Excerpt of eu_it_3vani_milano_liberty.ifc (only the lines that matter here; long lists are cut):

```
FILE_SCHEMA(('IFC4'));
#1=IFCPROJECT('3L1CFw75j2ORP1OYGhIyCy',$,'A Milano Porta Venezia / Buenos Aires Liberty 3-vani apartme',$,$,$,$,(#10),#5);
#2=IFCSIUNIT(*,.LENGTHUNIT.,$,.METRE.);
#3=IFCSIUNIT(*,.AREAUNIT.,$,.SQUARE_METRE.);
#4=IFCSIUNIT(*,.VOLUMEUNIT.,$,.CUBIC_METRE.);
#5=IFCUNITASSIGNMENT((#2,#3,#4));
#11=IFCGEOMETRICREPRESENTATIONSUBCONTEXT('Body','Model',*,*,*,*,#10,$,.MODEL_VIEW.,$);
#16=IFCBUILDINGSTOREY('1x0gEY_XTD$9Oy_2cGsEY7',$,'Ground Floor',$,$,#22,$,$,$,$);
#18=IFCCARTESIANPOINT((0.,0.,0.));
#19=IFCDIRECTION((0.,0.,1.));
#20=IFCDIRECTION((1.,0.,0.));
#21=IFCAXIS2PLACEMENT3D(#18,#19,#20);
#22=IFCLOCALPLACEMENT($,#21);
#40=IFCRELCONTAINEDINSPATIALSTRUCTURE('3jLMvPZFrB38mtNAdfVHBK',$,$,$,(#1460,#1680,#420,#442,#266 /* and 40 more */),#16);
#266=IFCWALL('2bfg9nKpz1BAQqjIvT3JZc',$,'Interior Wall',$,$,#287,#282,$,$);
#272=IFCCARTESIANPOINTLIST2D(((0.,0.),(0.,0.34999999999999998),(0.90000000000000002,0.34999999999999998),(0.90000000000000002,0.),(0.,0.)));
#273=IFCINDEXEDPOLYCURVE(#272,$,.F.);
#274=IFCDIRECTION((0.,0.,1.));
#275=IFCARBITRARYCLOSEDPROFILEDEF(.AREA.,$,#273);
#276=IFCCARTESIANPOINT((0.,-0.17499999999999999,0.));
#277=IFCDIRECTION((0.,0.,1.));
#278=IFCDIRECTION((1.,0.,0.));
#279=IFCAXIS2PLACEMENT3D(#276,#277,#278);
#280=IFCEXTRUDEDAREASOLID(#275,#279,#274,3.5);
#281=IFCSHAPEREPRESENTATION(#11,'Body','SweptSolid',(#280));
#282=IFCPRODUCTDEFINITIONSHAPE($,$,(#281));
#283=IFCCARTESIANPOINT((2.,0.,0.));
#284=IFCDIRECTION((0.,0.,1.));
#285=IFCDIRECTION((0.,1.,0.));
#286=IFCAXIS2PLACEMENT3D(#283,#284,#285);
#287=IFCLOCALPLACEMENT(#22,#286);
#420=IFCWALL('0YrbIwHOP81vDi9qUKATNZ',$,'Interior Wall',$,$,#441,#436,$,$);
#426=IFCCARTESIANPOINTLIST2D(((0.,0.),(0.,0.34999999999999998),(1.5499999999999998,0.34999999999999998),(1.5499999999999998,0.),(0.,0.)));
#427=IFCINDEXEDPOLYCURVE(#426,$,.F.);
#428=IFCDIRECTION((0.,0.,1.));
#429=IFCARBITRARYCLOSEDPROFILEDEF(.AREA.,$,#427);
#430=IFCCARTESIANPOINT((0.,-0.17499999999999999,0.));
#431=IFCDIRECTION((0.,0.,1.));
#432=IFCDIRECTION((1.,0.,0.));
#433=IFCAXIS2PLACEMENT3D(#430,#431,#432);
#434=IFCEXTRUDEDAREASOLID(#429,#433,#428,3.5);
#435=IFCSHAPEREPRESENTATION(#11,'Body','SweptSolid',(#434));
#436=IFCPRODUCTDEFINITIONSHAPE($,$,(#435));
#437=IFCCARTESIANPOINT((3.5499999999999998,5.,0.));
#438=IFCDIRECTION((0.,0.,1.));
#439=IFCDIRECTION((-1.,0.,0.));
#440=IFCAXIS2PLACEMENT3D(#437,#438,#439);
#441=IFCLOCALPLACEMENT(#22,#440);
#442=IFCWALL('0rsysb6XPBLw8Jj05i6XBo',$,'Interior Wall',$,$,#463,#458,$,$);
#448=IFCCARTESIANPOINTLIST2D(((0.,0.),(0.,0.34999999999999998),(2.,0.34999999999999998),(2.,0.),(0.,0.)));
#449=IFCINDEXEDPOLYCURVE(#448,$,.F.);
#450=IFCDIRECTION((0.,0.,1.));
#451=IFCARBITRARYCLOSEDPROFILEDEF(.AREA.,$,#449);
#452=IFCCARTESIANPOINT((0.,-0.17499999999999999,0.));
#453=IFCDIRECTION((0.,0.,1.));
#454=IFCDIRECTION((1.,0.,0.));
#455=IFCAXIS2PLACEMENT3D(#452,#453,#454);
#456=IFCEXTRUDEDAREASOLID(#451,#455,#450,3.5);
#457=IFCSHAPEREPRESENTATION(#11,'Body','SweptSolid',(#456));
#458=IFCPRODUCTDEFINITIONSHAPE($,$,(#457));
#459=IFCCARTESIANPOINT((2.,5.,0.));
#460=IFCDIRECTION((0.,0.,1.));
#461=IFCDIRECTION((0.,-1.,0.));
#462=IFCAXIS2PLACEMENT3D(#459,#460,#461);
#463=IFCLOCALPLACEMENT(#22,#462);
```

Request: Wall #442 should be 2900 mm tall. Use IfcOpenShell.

```python
import ifcopenshell
import ifcopenshell.geom
import ifcopenshell.util.representation
import ifcopenshell.util.shape

model = ifcopenshell.open("eu_it_3vani_milano_liberty.ifc")
settings = ifcopenshell.geom.settings()


def volume(element):
    """Net volume in cubic metres, openings subtracted."""
    shape = ifcopenshell.geom.create_shape(settings, element)
    return ifcopenshell.util.shape.get_volume(shape.geometry)


wall = model.by_id(442)
before = volume(wall)

body = ifcopenshell.util.representation.get_representation(wall, "Model", "Body")
solid = body.Items[0]
old_height = solid.Depth
solid.Depth = 2.9
after = volume(wall)

print(f"height {old_height:g} -> {solid.Depth:g}, volume {before:.3f} -> {after:.3f} m3")

model.write("eu_it_3vani_milano_liberty_updated.ifc")
```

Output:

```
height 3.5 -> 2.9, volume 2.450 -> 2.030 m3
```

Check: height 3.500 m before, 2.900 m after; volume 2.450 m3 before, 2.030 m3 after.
